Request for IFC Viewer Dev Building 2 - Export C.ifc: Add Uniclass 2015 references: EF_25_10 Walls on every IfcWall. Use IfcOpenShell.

First a look at what the model holds.

```python
import ifcopenshell

model = ifcopenshell.open("IFC Viewer Dev Building 2 - Export C.ifc")
print(model.schema)
print("classifications:", [c.Name for c in model.by_type("IfcClassification")])
for ifc_class in ("IfcDoor", "IfcRoof", "IfcStair", "IfcWall", "IfcWindow"):
    print(ifc_class, len(model.by_type(ifc_class)))
```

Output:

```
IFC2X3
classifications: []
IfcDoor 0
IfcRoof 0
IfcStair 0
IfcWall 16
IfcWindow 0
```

```python
import ifcopenshell
import ifcopenshell.api.classification

model = ifcopenshell.open("IFC Viewer Dev Building 2 - Export C.ifc")

# IFC2X3 requires Source and Edition and has no link from the project to the system.
system = model.create_entity("IfcClassification", Source="NBS", Edition="2015", Name="Uniclass 2015")

codes = {
    "IfcWall": ("EF_25_10", "Walls"),
}
for ifc_class, (code, name) in codes.items():
    products = model.by_type(ifc_class)
    ifcopenshell.api.classification.add_reference(
        model, products=products, classification=system, identification=code, name=name
    )
    print(code, len(products))

model.write("IFC Viewer Dev Building 2 - Export C_v2.ifc")
```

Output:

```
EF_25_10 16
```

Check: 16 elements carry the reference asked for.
